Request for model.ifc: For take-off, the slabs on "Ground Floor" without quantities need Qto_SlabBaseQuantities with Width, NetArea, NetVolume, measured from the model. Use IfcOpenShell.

First a look at what the model holds.

```python
import ifcopenshell
import ifcopenshell.util.element
import ifcopenshell.util.unit

model = ifcopenshell.open("model.ifc")
print(model.schema)
for unit_type in ("LENGTHUNIT", "AREAUNIT", "VOLUMEUNIT"):
    print(unit_type, ifcopenshell.util.unit.calculate_unit_scale(model, unit_type))
storey = next(s for s in model.by_type("IfcBuildingStorey") if s.Name == "Ground Floor")
slabs = [e for e in ifcopenshell.util.element.get_decomposition(storey) if e.is_a("IfcSlab")]
for e in sorted(slabs, key=lambda e: e.id()):
    print(e.id(), e.is_a(), e.Name, list(ifcopenshell.util.element.get_psets(e, qtos_only=True)), sep=" | ")
```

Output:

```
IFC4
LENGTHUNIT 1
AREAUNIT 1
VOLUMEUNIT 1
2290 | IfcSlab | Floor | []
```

```python
import ifcopenshell
import ifcopenshell.api.pset
import ifcopenshell.geom
import ifcopenshell.util.element
import ifcopenshell.util.shape
import ifcopenshell.util.unit

model = ifcopenshell.open("model.ifc")
unit_scale = ifcopenshell.util.unit.calculate_unit_scale(model)
area_scale = ifcopenshell.util.unit.calculate_unit_scale(model, "AREAUNIT")
volume_scale = ifcopenshell.util.unit.calculate_unit_scale(model, "VOLUMEUNIT")
settings = ifcopenshell.geom.settings()

storey = next(s for s in model.by_type("IfcBuildingStorey") if s.Name == "Ground Floor")
slabs = [e for e in ifcopenshell.util.element.get_decomposition(storey) if e.is_a("IfcSlab")]

for e in sorted(slabs, key=lambda e: e.id()):
    if ifcopenshell.util.element.get_psets(e, qtos_only=True, should_inherit=False):
        continue
    # Geometry comes back in metres, in the element's own axes.
    shape = ifcopenshell.geom.create_shape(settings, e)
    values = {
        "Width": ifcopenshell.util.shape.get_z(shape.geometry) / unit_scale,
        "NetArea": ifcopenshell.util.shape.get_footprint_area(shape.geometry) / area_scale,
        "NetVolume": ifcopenshell.util.shape.get_volume(shape.geometry) / volume_scale,
    }
    qto = ifcopenshell.api.pset.add_qto(model, product=e, name="Qto_SlabBaseQuantities")
    ifcopenshell.api.pset.edit_qto(model, qto=qto, properties=values)
    print(e.id(), {k: round(v, 3) for k, v in values.items()})

model.write("model_updated.ifc")
```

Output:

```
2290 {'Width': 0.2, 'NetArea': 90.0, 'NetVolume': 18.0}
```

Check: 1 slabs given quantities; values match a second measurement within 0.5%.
